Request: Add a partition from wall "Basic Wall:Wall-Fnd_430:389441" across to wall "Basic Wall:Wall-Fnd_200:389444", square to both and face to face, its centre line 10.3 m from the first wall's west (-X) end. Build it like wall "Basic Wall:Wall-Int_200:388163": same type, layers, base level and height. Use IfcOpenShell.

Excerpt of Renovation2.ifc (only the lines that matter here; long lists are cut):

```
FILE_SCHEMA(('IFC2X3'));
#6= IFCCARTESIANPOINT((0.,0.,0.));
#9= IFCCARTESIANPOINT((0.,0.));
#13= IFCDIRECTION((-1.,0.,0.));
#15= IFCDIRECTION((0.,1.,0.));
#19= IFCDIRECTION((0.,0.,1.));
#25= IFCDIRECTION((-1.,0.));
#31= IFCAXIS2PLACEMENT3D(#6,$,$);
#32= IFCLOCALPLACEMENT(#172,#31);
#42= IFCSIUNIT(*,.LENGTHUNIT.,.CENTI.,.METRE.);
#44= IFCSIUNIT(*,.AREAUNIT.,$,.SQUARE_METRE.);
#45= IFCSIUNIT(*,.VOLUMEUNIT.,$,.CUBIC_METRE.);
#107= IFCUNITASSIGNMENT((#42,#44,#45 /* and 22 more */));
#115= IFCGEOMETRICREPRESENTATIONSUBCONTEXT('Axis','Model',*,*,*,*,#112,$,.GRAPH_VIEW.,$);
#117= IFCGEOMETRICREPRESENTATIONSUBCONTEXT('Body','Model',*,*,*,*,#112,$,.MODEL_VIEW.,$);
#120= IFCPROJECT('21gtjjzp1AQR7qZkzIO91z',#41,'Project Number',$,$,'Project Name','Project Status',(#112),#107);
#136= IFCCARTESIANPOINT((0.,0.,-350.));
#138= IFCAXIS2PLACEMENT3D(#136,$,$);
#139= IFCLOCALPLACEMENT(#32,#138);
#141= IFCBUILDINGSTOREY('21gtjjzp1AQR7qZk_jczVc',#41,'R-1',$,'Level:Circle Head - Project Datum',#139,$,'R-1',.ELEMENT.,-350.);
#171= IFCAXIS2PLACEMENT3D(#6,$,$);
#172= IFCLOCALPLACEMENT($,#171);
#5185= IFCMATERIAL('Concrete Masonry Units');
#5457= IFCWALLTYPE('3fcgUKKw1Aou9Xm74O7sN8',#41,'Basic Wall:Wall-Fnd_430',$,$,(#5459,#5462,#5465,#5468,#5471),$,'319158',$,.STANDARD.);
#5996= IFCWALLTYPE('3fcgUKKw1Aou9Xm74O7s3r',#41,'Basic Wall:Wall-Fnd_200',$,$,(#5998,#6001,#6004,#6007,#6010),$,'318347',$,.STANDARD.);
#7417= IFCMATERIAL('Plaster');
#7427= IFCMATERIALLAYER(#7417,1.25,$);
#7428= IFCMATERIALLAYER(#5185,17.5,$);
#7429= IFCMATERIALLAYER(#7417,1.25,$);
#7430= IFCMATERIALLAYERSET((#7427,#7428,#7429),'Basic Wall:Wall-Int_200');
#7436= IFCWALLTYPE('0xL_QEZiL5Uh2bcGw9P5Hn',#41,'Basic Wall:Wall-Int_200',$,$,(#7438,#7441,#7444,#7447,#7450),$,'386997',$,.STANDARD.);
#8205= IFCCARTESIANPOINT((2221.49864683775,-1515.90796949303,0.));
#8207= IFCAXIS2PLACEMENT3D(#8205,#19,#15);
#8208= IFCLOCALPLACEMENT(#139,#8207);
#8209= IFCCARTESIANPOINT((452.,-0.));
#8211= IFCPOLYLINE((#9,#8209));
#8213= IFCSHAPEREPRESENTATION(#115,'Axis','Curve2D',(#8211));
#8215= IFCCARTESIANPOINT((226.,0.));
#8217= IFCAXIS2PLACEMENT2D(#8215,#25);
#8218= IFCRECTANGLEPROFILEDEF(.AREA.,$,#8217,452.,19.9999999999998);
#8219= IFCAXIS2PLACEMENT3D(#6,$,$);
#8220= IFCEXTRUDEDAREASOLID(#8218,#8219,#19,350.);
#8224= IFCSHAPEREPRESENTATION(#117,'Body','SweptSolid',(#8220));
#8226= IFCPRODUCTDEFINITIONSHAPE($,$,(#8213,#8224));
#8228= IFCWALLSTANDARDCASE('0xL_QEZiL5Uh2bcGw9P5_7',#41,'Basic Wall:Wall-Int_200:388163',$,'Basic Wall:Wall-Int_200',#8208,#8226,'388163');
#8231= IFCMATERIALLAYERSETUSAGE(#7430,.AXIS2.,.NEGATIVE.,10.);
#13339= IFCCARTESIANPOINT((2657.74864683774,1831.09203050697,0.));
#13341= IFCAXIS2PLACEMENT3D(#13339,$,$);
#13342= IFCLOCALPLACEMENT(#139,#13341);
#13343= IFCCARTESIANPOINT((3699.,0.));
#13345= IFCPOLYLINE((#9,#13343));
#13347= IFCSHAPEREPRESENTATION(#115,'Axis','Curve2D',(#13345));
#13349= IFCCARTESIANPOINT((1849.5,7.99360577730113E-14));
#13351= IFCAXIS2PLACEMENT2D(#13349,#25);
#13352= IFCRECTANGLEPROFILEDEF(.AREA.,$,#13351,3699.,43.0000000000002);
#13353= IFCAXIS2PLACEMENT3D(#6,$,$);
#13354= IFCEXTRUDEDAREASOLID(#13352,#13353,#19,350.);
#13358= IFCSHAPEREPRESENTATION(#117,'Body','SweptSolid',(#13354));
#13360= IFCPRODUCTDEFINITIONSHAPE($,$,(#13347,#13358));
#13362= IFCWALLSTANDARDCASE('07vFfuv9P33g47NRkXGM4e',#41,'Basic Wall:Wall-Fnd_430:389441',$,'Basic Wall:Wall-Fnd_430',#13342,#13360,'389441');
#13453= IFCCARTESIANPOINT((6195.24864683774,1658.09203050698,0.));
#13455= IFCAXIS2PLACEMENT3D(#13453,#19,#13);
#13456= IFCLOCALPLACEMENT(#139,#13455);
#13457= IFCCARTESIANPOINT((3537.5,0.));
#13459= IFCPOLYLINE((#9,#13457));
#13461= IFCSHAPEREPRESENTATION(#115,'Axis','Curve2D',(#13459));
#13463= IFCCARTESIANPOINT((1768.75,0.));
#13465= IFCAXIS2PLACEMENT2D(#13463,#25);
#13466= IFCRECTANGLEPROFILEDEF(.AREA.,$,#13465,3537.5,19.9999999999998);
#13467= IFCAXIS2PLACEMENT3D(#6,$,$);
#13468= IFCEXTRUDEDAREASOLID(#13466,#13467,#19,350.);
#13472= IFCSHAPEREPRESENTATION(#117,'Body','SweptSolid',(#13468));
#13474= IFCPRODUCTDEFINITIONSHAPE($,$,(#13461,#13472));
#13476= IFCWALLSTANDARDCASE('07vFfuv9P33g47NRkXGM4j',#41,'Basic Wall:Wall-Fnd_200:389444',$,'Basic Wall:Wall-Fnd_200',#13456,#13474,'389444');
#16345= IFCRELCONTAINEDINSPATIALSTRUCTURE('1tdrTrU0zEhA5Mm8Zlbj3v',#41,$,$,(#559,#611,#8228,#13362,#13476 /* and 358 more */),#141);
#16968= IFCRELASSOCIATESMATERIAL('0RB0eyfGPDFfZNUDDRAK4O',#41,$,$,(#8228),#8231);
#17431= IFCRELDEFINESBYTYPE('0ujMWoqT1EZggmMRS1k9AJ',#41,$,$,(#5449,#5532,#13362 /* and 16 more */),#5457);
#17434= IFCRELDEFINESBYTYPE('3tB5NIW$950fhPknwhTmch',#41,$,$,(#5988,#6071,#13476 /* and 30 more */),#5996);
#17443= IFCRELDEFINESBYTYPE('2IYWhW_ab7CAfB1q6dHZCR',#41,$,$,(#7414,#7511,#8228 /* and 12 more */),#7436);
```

```python
import numpy as np
import ifcopenshell
import ifcopenshell.api.geometry
import ifcopenshell.api.material
import ifcopenshell.api.pset
import ifcopenshell.api.root
import ifcopenshell.api.spatial
import ifcopenshell.api.type
import ifcopenshell.geom
import ifcopenshell.util.element
import ifcopenshell.util.placement
import ifcopenshell.util.representation
import ifcopenshell.util.shape
import ifcopenshell.util.unit

model = ifcopenshell.open("Renovation2.ifc")
unit_scale = ifcopenshell.util.unit.calculate_unit_scale(model)
settings = ifcopenshell.geom.settings()
settings.set("use-world-coords", True)

start_wall = model.by_guid("07vFfuv9P33g47NRkXGM4e")
end_wall = model.by_guid("07vFfuv9P33g47NRkXGM4j")
like = model.by_guid("0xL_QEZiL5Uh2bcGw9P5_7")
matrix = ifcopenshell.util.placement.get_local_placement(start_wall.ObjectPlacement)
matrix[:3, 3] *= unit_scale


def extent(element):
    """Bounding box in the first wall's axes, in metres."""
    shape = ifcopenshell.geom.create_shape(settings, element)
    points = (ifcopenshell.util.shape.get_vertices(shape.geometry) - matrix[:3, 3]) @ matrix[:3, :3]
    return points.min(axis=0), points.max(axis=0)


y_start = extent(start_wall)[0][1]
y_end = extent(end_wall)[1][1]
like_min, like_max = extent(like)
length, height = float(abs(y_end - y_start)), float(like_max[2] - like_min[2])
layer_set = ifcopenshell.util.element.get_material(like, should_skip_usage=True)
thickness = sum(layer.LayerThickness for layer in layer_set.MaterialLayers) * unit_scale

wall = ifcopenshell.api.root.create_entity(model, ifc_class="IfcWallStandardCase", name="New partition")
storey = ifcopenshell.util.element.get_container(like)
ifcopenshell.api.spatial.assign_container(model, products=[wall], relating_structure=storey)
ifcopenshell.api.type.assign_type(
    model, related_objects=[wall], relating_type=ifcopenshell.util.element.get_type(like), should_map_representations=False
)
rel = ifcopenshell.api.material.assign_material(
    model, products=[wall], type="IfcMaterialLayerSetUsage", material=layer_set
)
rel.RelatingMaterial.OffsetFromReferenceLine = -thickness / 2 / unit_scale
pset = ifcopenshell.api.pset.add_pset(model, product=wall, name="Pset_WallCommon")
ifcopenshell.api.pset.edit_pset(model, pset=pset, properties={"IsExternal": False, "LoadBearing": False})

# The axis runs down the middle of the wall.
axis = ifcopenshell.api.geometry.add_axis_representation(
    model, context=ifcopenshell.util.representation.get_context(model, "Model", "Axis"), axis=[(0.0, 0.0), (length, 0.0)]
)
body = ifcopenshell.api.geometry.add_wall_representation(
    model,
    context=ifcopenshell.util.representation.get_context(model, "Model", "Body", "MODEL_VIEW"),
    length=length,
    height=height,
    thickness=thickness,
    offset=-thickness / 2,
)
for representation in (axis, body):
    ifcopenshell.api.geometry.assign_representation(model, product=wall, representation=representation)

placement = matrix @ ifcopenshell.util.placement.rotation(-90, "Z")
placement[:, 3] = matrix @ np.array([extent(start_wall)[0][0] + 10.3, y_start, like_min[2], 1.0])
ifcopenshell.api.geometry.edit_object_placement(model, product=wall, matrix=placement)

print(f"partition {length:.3f} m long, {height:.3f} m high, {thickness:.3f} m thick")

model.write("Renovation2_rev.ifc")
```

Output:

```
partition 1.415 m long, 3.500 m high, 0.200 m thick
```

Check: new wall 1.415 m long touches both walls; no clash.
